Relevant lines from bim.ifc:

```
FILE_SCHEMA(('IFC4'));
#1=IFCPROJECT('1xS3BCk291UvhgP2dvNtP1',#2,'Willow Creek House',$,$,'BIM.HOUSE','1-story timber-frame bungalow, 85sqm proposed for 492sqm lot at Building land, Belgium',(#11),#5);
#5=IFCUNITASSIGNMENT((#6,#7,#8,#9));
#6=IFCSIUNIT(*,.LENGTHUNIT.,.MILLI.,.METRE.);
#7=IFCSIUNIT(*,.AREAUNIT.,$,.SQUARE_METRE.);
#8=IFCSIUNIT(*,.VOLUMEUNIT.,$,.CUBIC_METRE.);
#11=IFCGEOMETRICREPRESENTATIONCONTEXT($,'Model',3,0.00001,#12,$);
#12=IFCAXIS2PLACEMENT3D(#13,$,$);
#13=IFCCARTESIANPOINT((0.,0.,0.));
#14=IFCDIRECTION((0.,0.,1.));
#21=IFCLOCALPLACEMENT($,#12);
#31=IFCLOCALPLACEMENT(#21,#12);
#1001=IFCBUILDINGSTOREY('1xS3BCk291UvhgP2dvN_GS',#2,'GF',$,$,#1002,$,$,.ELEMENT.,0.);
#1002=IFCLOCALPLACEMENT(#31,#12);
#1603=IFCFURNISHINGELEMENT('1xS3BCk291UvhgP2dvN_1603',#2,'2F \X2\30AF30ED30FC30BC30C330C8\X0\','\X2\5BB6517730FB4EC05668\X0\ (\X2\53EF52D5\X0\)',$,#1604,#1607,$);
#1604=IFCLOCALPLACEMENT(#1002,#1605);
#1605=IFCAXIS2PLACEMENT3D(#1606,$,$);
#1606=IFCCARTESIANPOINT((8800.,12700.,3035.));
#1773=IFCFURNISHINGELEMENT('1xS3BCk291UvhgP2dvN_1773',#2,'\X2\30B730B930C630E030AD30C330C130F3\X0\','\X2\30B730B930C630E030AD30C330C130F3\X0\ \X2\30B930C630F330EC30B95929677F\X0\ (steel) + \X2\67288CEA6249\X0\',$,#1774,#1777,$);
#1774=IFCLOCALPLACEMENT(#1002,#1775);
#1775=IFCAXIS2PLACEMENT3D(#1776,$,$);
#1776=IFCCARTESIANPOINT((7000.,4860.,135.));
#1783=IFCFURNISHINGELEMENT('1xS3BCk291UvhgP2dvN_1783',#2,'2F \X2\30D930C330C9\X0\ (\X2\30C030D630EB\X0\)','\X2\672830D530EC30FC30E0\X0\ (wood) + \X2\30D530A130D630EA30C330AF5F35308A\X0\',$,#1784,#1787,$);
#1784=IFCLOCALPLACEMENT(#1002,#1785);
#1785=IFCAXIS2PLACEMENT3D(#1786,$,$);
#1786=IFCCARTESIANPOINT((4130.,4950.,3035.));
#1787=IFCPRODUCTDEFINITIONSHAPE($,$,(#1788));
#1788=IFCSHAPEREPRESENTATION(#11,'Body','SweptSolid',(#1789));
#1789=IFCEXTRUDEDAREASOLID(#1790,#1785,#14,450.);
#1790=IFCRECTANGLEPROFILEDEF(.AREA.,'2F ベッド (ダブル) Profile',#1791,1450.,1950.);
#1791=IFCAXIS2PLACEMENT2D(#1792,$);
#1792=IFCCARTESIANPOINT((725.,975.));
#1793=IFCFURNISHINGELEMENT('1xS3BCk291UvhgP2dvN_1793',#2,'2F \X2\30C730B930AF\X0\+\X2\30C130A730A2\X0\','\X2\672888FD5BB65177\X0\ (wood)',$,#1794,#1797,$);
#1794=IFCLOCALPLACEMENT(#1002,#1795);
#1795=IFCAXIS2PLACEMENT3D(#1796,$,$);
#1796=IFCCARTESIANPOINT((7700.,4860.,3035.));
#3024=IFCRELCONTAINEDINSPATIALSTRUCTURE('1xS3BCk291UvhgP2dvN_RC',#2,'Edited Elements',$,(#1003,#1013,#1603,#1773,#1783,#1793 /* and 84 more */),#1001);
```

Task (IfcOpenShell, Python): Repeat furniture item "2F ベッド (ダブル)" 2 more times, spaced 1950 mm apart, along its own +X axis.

```python
import ifcopenshell
import ifcopenshell.api.geometry
import ifcopenshell.api.root
import ifcopenshell.util.element
import ifcopenshell.util.placement
import ifcopenshell.util.unit

model = ifcopenshell.open("bim.ifc")
unit_scale = ifcopenshell.util.unit.calculate_unit_scale(model)


def reuse_history(source, copy):
    """copy_class also copies each property set's owner history, people and application; keep the originals."""
    for rel in copy.IsDefinedBy:
        if rel.is_a("IfcRelDefinesByProperties") and (history := rel.RelatingPropertyDefinition.OwnerHistory):
            rel.RelatingPropertyDefinition.OwnerHistory = source.OwnerHistory
            ifcopenshell.util.element.remove_deep2(model, history)


source = model.by_id(1783)
base = ifcopenshell.util.placement.get_local_placement(source.ObjectPlacement)
step = base[:3, 0] * 1.95 / unit_scale

for i in range(1, 3):
    copy = ifcopenshell.api.root.copy_class(model, product=source)
    copy.Representation = ifcopenshell.util.element.copy_deep(
        model, source.Representation, exclude=["IfcGeometricRepresentationContext", "IfcRepresentationMap"]
    )
    reuse_history(source, copy)
    matrix = base.copy()
    matrix[:3, 3] += i * step
    print("added at", matrix[:3, 3].round(3) + 0.0)
    ifcopenshell.api.geometry.edit_object_placement(model, product=copy, matrix=matrix, is_si=False)

model.write("bim_v2.ifc")
```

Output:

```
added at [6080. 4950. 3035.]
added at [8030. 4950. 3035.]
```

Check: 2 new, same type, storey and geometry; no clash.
